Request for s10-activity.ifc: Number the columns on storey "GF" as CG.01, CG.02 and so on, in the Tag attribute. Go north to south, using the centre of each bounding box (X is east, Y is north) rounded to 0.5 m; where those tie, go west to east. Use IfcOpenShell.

First a look at what the model holds.

```python
import ifcopenshell
import ifcopenshell.util.element
import ifcopenshell.util.placement

model = ifcopenshell.open("s10-activity.ifc")
print(model.schema)
storey = next(s for s in model.by_type("IfcBuildingStorey") if s.Name == "GF")
columns = [e for e in ifcopenshell.util.element.get_decomposition(storey) if e.is_a("IfcColumn")]
for e in sorted(columns, key=lambda e: e.id()):
    origin = ifcopenshell.util.placement.get_local_placement(e.ObjectPlacement)[:3, 3]
    print(e.id(), e.Tag, e.Name, origin.round(2) + 0.0, sep=" | ")
```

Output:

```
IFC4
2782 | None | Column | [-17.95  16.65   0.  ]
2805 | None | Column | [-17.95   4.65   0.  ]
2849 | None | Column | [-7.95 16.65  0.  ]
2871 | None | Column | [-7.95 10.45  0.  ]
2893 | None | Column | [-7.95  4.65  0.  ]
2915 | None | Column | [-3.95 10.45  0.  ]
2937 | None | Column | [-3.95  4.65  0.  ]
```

```python
import ifcopenshell
import ifcopenshell.geom
import ifcopenshell.util.element
import ifcopenshell.util.shape

model = ifcopenshell.open("s10-activity.ifc")
settings = ifcopenshell.geom.settings()
settings.set("use-world-coords", True)


def centre(element):
    shape = ifcopenshell.geom.create_shape(settings, element)
    return ifcopenshell.util.shape.get_bbox_centroid(shape.geometry)


storey = next(s for s in model.by_type("IfcBuildingStorey") if s.Name == "GF")
columns = [e for e in ifcopenshell.util.element.get_decomposition(storey) if e.is_a("IfcColumn")]

# Insertion points can sit at a corner or the storey origin, so sort by the geometry (in metres).
centres = {e: centre(e) for e in columns}
columns.sort(key=lambda e: (-round(centres[e][1] / 0.5), centres[e][0]))

for i, e in enumerate(columns, start=1):
    number = f"CG.{i:02d}"
    e.Tag = number
    print(e.id(), number)

model.write("s10-activity_updated.ifc")
```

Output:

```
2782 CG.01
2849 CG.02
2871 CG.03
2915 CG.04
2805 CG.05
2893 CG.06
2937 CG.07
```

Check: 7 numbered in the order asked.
